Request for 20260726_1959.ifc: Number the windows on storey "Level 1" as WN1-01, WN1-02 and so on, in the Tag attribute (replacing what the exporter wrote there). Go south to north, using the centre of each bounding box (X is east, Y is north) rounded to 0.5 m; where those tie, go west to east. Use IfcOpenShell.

First a look at what the model holds.

```python
import ifcopenshell
import ifcopenshell.util.element
import ifcopenshell.util.placement

model = ifcopenshell.open("20260726_1959.ifc")
print(model.schema)
storey = next(s for s in model.by_type("IfcBuildingStorey") if s.Name == "Level 1")
windows = [e for e in ifcopenshell.util.element.get_decomposition(storey) if e.is_a("IfcWindow")]
for e in sorted(windows, key=lambda e: e.id()):
    origin = ifcopenshell.util.placement.get_local_placement(e.ObjectPlacement)[:3, 3]
    print(e.id(), e.Tag, e.Name, origin.round(2) + 0.0, sep=" | ")
```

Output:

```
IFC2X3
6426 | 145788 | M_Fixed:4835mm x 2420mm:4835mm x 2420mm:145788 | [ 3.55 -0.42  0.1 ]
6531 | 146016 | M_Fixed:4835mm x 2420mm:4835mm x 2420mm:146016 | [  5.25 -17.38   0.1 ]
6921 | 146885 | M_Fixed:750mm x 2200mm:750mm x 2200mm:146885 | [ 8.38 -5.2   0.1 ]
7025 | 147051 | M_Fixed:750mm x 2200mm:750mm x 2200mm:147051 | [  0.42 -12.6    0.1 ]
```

```python
import ifcopenshell
import ifcopenshell.geom
import ifcopenshell.util.element
import ifcopenshell.util.shape

model = ifcopenshell.open("20260726_1959.ifc")
settings = ifcopenshell.geom.settings()
settings.set("use-world-coords", True)


def centre(element):
    shape = ifcopenshell.geom.create_shape(settings, element)
    return ifcopenshell.util.shape.get_bbox_centroid(shape.geometry)


storey = next(s for s in model.by_type("IfcBuildingStorey") if s.Name == "Level 1")
windows = [e for e in ifcopenshell.util.element.get_decomposition(storey) if e.is_a("IfcWindow")]

# Insertion points can sit at a corner or the storey origin, so sort by the geometry (in metres).
centres = {e: centre(e) for e in windows}
windows.sort(key=lambda e: (round(centres[e][1] / 0.5), centres[e][0]))

for i, e in enumerate(windows, start=1):
    number = f"WN1-{i:02d}"
    e.Tag = number
    print(e.id(), number)

model.write("20260726_1959_edited.ifc")
```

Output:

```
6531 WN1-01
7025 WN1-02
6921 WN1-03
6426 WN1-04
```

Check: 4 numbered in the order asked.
